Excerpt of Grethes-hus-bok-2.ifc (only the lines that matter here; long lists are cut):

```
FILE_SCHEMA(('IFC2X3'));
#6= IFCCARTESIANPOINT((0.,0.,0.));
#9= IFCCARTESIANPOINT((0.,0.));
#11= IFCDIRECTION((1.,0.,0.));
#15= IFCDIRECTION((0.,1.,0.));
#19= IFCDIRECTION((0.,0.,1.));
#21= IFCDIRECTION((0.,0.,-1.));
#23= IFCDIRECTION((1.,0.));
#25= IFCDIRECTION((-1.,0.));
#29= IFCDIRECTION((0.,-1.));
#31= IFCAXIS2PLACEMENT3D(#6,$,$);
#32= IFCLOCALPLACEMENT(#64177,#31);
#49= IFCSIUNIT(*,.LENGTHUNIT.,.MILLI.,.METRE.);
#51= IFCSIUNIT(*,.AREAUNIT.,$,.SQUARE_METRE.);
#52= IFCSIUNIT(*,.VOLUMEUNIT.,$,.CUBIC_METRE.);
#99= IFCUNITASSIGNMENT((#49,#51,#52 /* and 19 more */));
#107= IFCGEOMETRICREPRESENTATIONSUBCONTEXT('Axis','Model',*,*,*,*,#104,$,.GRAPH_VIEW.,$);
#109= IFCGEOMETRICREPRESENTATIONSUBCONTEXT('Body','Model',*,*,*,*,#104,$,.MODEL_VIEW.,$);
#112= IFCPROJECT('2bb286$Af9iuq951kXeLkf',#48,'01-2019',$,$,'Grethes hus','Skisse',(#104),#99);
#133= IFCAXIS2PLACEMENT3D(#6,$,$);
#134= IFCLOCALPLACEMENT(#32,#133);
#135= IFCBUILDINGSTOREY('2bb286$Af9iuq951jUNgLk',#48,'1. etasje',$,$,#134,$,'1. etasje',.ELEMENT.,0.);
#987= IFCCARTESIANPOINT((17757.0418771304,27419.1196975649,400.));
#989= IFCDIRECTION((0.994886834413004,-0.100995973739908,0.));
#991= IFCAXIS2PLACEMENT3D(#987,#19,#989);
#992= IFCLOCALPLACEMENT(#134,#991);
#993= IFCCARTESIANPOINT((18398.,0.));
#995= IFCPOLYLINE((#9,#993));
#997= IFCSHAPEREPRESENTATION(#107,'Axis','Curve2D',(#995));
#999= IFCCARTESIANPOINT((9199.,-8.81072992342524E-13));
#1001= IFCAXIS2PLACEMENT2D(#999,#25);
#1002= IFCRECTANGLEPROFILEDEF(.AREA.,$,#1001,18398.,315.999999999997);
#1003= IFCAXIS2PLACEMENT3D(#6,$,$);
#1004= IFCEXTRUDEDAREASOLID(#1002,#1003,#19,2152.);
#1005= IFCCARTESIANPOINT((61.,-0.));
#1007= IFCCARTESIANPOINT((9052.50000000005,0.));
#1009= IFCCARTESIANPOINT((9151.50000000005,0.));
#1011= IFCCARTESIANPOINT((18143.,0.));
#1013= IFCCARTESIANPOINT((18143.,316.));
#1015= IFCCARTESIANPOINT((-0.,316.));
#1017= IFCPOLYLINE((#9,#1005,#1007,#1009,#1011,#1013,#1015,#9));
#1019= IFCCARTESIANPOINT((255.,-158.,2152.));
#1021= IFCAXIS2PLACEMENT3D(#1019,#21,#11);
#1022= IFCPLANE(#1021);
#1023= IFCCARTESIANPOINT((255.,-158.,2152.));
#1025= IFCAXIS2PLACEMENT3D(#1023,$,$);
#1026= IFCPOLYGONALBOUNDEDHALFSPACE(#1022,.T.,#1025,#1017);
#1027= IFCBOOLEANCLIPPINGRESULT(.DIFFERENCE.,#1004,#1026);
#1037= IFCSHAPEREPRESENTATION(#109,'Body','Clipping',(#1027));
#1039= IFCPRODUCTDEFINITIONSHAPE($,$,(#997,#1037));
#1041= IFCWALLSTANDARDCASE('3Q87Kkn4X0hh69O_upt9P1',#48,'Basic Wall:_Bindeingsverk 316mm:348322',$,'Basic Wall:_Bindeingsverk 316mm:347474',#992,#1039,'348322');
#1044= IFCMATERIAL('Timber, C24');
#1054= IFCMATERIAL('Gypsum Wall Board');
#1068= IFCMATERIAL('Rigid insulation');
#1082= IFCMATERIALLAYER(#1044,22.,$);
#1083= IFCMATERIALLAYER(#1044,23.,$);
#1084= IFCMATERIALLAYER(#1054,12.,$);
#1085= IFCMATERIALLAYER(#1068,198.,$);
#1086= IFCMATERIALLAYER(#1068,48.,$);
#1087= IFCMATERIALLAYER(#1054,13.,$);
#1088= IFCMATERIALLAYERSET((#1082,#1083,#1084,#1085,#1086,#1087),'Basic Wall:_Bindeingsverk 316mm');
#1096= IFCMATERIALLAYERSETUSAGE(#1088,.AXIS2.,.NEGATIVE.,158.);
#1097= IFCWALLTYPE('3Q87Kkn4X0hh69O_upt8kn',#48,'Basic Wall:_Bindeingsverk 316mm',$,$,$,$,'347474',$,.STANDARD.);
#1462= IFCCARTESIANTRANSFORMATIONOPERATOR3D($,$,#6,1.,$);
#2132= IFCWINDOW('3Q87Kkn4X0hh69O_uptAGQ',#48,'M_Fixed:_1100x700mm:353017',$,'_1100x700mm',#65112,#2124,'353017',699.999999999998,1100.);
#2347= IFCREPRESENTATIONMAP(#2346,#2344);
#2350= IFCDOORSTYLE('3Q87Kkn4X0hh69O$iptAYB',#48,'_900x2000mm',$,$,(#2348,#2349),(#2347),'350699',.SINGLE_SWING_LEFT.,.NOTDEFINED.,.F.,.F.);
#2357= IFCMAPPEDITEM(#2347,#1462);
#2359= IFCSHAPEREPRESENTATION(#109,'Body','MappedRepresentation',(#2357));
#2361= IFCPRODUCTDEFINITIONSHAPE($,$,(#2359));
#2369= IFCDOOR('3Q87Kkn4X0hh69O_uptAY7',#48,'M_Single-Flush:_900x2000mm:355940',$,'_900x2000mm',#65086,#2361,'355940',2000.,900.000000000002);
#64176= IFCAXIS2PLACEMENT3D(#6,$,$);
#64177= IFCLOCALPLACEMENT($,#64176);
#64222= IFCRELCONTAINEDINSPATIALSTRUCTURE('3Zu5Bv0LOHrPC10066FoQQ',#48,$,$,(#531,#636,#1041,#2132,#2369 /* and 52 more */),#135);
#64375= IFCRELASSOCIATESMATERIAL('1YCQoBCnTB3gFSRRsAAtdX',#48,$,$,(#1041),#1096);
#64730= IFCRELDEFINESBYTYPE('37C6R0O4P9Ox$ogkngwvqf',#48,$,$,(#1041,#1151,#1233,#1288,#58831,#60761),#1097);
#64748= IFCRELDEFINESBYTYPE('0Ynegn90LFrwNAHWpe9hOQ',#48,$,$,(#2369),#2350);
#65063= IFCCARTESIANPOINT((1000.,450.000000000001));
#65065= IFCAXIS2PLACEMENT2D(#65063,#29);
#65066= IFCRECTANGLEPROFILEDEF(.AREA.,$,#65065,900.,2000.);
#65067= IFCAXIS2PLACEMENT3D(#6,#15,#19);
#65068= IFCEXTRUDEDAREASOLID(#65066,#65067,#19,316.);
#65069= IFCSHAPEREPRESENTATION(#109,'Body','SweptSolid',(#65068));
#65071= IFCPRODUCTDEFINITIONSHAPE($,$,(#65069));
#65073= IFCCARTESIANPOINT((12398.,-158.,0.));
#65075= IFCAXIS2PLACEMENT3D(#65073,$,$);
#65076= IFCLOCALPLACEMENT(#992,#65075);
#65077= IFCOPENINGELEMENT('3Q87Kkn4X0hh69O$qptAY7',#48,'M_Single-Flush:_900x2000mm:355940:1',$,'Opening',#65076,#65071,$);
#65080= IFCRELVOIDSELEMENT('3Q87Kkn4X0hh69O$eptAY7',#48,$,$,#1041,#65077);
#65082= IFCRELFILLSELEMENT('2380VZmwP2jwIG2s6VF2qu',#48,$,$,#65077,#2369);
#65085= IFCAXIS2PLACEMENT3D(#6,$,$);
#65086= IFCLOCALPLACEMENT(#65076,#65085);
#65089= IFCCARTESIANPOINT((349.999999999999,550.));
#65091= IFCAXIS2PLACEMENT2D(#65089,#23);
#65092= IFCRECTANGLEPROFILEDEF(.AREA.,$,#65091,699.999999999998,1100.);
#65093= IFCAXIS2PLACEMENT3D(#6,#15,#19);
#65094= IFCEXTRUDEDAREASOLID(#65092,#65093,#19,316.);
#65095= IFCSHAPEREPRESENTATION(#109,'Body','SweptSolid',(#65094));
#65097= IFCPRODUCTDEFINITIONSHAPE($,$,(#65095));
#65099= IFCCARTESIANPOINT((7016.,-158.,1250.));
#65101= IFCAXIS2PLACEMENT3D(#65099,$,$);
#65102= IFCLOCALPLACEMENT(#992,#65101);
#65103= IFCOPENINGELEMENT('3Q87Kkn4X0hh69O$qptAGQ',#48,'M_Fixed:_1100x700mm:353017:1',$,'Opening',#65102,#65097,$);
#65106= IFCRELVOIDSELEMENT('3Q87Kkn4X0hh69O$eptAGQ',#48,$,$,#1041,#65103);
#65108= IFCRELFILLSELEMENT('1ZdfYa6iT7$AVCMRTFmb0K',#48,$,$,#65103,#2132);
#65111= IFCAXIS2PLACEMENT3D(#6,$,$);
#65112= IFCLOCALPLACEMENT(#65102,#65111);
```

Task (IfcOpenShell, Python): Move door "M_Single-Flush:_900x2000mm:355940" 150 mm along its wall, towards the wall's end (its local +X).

```python
import ifcopenshell
import ifcopenshell.api.geometry
import ifcopenshell.util.placement
import ifcopenshell.util.unit

model = ifcopenshell.open("Grethes-hus-bok-2.ifc")
unit_scale = ifcopenshell.util.unit.calculate_unit_scale(model)

door = model.by_guid("3Q87Kkn4X0hh69O_uptAY7")
opening = door.FillsVoids[0].RelatingOpeningElement
wall = opening.VoidsElements[0].RelatingBuildingElement

wall_matrix = ifcopenshell.util.placement.get_local_placement(wall.ObjectPlacement)
shift = wall_matrix[:3, 0] * 0.15 / unit_scale
before = ifcopenshell.util.placement.get_local_placement(door.ObjectPlacement)[:3, 3].copy()

# The door is placed relative to its opening, so it follows when the opening moves.
matrix = ifcopenshell.util.placement.get_local_placement(opening.ObjectPlacement)
matrix[:3, 3] += shift
ifcopenshell.api.geometry.edit_object_placement(
    model, product=opening, matrix=matrix, is_si=False, should_transform_children=True
)

after = ifcopenshell.util.placement.get_local_placement(door.ObjectPlacement)[:3, 3]
print("door moved by", (after - before).round(3) + 0.0)

model.write("Grethes-hus-bok-2_rev.ifc")
```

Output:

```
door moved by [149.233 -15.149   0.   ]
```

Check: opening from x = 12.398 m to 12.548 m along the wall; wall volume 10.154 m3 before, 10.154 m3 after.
